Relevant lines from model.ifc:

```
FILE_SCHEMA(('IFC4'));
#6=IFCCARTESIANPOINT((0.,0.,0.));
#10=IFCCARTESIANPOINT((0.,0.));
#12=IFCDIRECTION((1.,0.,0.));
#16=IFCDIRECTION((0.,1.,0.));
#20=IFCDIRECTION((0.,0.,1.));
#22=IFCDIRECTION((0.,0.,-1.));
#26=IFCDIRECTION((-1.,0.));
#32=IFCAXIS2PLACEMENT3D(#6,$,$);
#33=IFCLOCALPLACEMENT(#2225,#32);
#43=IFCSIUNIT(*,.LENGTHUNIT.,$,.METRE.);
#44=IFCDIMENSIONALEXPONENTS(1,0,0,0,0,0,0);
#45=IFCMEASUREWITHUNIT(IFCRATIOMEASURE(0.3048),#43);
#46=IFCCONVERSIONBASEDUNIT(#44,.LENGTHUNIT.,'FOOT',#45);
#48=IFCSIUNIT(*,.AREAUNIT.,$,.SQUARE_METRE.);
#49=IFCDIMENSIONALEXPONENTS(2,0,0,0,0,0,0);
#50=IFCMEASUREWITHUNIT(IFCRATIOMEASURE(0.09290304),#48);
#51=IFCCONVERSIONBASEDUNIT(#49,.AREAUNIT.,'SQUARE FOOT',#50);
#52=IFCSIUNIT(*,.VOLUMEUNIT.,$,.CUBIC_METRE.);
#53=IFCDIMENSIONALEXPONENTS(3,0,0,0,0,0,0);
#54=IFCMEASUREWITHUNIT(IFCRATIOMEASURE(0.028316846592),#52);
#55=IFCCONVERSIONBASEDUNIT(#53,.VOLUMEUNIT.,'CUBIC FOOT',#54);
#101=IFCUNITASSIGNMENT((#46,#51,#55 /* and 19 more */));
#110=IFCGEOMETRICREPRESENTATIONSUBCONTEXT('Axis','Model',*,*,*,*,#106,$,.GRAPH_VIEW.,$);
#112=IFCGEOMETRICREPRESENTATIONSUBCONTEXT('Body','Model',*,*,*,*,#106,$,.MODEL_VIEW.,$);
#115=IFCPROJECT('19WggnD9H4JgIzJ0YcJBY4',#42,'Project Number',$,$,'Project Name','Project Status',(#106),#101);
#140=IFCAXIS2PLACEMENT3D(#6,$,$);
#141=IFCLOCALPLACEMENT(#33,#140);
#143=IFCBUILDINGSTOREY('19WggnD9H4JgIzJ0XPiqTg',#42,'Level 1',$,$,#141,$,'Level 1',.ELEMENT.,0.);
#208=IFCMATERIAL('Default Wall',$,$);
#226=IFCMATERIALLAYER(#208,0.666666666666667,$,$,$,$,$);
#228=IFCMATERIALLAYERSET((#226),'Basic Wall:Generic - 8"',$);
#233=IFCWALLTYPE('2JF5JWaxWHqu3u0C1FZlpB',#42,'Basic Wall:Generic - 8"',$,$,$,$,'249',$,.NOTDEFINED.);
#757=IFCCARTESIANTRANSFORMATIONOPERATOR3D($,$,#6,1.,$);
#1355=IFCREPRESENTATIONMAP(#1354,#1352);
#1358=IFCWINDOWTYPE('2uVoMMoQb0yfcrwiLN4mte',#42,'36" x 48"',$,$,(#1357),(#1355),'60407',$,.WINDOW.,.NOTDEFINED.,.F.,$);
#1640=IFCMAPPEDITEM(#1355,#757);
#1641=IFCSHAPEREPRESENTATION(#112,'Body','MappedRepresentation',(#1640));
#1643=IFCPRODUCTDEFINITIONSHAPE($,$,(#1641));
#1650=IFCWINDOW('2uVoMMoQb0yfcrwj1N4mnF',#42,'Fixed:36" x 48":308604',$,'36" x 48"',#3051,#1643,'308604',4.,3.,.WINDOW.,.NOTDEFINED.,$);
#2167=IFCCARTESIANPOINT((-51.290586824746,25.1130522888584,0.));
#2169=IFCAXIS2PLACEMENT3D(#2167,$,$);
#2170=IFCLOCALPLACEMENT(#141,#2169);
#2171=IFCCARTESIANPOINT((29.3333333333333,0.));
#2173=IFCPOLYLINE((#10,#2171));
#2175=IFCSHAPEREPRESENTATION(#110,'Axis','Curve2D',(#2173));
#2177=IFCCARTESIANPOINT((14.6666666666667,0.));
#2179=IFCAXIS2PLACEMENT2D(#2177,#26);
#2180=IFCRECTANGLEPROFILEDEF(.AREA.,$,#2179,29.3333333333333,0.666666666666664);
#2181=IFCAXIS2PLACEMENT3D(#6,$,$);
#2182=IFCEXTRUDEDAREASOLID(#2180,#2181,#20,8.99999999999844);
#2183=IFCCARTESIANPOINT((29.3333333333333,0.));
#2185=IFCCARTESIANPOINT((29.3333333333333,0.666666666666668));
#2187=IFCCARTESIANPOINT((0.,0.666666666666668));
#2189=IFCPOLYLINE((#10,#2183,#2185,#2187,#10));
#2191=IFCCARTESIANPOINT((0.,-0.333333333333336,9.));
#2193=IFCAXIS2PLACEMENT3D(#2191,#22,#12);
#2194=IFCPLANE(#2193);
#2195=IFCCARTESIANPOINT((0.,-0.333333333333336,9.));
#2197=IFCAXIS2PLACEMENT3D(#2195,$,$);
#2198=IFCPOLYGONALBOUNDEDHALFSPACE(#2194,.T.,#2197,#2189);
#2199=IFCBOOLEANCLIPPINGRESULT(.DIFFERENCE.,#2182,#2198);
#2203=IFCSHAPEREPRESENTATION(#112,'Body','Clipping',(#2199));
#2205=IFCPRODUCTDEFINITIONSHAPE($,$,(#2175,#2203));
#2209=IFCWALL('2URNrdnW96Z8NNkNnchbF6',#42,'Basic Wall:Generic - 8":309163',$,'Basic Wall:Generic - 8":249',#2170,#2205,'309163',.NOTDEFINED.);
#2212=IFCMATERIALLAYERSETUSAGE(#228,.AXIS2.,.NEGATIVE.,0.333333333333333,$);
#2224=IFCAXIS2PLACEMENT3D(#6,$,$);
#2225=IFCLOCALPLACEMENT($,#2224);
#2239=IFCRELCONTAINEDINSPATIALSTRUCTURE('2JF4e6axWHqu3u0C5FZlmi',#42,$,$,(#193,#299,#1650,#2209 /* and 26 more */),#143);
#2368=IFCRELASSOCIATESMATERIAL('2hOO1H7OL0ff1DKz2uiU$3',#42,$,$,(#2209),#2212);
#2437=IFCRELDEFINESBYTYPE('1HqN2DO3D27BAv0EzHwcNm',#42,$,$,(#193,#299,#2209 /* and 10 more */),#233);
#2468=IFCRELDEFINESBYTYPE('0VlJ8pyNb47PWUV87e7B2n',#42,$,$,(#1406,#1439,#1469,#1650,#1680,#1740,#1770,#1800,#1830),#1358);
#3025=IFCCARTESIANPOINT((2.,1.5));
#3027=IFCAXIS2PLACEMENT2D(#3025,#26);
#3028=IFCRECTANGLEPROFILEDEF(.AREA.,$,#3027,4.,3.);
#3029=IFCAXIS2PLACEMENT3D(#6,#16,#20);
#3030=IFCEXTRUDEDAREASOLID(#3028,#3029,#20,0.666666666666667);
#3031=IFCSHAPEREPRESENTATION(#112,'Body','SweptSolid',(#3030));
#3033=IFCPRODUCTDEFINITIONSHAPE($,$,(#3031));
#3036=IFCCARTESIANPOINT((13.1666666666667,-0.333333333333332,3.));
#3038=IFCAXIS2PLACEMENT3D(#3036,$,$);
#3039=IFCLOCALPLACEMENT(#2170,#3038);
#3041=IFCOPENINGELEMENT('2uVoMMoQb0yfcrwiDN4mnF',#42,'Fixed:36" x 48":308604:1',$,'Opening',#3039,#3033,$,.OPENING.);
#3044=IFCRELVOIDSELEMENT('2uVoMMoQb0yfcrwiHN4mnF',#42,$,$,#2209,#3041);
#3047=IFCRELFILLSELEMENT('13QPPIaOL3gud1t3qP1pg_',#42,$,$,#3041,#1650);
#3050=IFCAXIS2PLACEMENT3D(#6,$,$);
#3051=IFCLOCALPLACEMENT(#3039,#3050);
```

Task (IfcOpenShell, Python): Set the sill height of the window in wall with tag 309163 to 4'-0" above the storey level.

```python
import numpy as np
import ifcopenshell
import ifcopenshell.api.geometry
import ifcopenshell.geom
import ifcopenshell.util.element
import ifcopenshell.util.placement
import ifcopenshell.util.shape
import ifcopenshell.util.unit

model = ifcopenshell.open("model.ifc")
unit_scale = ifcopenshell.util.unit.calculate_unit_scale(model)

window = model.by_guid("2uVoMMoQb0yfcrwj1N4mnF")
opening = window.FillsVoids[0].RelatingOpeningElement
storey = ifcopenshell.util.element.get_container(window, ifc_class="IfcBuildingStorey")
level = ifcopenshell.util.placement.get_local_placement(storey.ObjectPlacement)[2, 3]

# The opening's origin need not be at the sill, so measure its lowest point.
shape = ifcopenshell.geom.create_shape(ifcopenshell.geom.settings(), opening)
bottom = ifcopenshell.util.shape.get_shape_bottom_elevation(shape, shape.geometry) / unit_scale
dz = level + 48 * 0.0254 / unit_scale - bottom

shift = np.array([0.0, 0.0, dz])
# The window is placed relative to its opening, so it follows when the opening moves.
matrix = ifcopenshell.util.placement.get_local_placement(opening.ObjectPlacement)
matrix[:3, 3] += shift
ifcopenshell.api.geometry.edit_object_placement(
    model, product=opening, matrix=matrix, is_si=False, should_transform_children=True
)

print(f"moved by {dz * unit_scale:+.3f} m")

model.write("model_rev.ifc")
```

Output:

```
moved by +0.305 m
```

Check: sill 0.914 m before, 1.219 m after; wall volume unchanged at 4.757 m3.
